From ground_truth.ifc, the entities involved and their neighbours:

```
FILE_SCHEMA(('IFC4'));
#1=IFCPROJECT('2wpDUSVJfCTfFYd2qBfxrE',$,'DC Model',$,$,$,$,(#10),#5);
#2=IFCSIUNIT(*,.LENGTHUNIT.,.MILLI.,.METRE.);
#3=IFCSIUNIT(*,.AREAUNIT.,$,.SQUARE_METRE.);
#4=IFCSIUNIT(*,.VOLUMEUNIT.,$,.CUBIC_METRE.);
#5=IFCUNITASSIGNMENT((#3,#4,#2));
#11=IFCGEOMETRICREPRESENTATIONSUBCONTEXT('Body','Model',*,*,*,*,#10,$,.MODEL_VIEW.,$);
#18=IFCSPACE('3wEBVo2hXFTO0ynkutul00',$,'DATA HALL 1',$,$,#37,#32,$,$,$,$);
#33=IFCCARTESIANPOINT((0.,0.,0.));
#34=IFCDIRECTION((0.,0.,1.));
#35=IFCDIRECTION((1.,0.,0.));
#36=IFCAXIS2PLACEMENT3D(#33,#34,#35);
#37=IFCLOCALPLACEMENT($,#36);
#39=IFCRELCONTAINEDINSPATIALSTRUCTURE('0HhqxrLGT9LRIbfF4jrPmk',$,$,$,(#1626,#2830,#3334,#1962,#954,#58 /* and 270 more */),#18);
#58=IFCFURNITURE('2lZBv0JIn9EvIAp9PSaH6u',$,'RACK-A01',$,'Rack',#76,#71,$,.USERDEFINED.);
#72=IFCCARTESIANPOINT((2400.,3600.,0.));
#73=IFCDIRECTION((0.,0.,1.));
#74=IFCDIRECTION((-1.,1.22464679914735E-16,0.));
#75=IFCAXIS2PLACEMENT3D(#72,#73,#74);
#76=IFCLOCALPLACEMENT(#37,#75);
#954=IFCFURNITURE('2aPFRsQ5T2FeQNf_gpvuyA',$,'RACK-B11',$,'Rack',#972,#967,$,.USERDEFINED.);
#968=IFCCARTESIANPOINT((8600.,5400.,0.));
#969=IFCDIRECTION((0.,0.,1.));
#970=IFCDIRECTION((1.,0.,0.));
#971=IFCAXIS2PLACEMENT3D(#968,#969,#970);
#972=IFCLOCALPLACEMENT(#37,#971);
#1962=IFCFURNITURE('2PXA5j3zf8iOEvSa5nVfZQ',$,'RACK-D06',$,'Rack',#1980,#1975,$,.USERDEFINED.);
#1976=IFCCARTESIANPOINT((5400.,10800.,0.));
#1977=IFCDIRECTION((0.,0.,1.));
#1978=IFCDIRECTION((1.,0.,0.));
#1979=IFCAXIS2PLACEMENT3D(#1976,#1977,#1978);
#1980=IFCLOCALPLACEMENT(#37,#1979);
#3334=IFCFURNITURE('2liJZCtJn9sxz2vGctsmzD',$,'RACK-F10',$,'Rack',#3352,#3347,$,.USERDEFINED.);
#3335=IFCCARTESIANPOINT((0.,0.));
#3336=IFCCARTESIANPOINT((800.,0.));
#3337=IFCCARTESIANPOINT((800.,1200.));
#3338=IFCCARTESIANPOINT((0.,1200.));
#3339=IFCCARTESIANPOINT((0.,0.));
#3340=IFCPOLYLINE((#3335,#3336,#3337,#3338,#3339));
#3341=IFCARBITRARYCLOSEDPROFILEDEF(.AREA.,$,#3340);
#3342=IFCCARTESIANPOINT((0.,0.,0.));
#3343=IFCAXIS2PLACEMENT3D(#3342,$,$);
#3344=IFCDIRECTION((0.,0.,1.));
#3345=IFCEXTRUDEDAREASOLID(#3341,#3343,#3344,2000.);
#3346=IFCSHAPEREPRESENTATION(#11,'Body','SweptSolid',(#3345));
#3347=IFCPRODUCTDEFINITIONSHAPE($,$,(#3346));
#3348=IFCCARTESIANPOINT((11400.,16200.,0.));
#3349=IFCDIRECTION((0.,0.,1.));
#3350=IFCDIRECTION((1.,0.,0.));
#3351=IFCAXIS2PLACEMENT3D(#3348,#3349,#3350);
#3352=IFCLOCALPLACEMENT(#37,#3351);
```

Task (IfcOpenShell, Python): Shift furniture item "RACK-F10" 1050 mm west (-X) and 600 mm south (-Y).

```python
import ifcopenshell
import ifcopenshell.api.geometry
import ifcopenshell.util.placement
import ifcopenshell.util.unit

model = ifcopenshell.open("ground_truth.ifc")
unit_scale = ifcopenshell.util.unit.calculate_unit_scale(model)

item = model.by_guid("2liJZCtJn9sxz2vGctsmzD")
matrix = ifcopenshell.util.placement.get_local_placement(item.ObjectPlacement)
matrix[0, 3] -= 1.05 / unit_scale
matrix[1, 3] -= 0.6 / unit_scale
ifcopenshell.api.geometry.edit_object_placement(model, product=item, matrix=matrix, is_si=False)

print(ifcopenshell.util.placement.get_local_placement(item.ObjectPlacement).round(3) + 0.0)

model.write("ground_truth_edited.ifc")
```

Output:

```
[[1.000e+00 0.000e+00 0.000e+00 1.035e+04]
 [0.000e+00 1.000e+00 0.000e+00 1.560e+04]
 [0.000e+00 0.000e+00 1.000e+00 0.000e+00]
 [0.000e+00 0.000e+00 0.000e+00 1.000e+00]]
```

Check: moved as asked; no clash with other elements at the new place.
